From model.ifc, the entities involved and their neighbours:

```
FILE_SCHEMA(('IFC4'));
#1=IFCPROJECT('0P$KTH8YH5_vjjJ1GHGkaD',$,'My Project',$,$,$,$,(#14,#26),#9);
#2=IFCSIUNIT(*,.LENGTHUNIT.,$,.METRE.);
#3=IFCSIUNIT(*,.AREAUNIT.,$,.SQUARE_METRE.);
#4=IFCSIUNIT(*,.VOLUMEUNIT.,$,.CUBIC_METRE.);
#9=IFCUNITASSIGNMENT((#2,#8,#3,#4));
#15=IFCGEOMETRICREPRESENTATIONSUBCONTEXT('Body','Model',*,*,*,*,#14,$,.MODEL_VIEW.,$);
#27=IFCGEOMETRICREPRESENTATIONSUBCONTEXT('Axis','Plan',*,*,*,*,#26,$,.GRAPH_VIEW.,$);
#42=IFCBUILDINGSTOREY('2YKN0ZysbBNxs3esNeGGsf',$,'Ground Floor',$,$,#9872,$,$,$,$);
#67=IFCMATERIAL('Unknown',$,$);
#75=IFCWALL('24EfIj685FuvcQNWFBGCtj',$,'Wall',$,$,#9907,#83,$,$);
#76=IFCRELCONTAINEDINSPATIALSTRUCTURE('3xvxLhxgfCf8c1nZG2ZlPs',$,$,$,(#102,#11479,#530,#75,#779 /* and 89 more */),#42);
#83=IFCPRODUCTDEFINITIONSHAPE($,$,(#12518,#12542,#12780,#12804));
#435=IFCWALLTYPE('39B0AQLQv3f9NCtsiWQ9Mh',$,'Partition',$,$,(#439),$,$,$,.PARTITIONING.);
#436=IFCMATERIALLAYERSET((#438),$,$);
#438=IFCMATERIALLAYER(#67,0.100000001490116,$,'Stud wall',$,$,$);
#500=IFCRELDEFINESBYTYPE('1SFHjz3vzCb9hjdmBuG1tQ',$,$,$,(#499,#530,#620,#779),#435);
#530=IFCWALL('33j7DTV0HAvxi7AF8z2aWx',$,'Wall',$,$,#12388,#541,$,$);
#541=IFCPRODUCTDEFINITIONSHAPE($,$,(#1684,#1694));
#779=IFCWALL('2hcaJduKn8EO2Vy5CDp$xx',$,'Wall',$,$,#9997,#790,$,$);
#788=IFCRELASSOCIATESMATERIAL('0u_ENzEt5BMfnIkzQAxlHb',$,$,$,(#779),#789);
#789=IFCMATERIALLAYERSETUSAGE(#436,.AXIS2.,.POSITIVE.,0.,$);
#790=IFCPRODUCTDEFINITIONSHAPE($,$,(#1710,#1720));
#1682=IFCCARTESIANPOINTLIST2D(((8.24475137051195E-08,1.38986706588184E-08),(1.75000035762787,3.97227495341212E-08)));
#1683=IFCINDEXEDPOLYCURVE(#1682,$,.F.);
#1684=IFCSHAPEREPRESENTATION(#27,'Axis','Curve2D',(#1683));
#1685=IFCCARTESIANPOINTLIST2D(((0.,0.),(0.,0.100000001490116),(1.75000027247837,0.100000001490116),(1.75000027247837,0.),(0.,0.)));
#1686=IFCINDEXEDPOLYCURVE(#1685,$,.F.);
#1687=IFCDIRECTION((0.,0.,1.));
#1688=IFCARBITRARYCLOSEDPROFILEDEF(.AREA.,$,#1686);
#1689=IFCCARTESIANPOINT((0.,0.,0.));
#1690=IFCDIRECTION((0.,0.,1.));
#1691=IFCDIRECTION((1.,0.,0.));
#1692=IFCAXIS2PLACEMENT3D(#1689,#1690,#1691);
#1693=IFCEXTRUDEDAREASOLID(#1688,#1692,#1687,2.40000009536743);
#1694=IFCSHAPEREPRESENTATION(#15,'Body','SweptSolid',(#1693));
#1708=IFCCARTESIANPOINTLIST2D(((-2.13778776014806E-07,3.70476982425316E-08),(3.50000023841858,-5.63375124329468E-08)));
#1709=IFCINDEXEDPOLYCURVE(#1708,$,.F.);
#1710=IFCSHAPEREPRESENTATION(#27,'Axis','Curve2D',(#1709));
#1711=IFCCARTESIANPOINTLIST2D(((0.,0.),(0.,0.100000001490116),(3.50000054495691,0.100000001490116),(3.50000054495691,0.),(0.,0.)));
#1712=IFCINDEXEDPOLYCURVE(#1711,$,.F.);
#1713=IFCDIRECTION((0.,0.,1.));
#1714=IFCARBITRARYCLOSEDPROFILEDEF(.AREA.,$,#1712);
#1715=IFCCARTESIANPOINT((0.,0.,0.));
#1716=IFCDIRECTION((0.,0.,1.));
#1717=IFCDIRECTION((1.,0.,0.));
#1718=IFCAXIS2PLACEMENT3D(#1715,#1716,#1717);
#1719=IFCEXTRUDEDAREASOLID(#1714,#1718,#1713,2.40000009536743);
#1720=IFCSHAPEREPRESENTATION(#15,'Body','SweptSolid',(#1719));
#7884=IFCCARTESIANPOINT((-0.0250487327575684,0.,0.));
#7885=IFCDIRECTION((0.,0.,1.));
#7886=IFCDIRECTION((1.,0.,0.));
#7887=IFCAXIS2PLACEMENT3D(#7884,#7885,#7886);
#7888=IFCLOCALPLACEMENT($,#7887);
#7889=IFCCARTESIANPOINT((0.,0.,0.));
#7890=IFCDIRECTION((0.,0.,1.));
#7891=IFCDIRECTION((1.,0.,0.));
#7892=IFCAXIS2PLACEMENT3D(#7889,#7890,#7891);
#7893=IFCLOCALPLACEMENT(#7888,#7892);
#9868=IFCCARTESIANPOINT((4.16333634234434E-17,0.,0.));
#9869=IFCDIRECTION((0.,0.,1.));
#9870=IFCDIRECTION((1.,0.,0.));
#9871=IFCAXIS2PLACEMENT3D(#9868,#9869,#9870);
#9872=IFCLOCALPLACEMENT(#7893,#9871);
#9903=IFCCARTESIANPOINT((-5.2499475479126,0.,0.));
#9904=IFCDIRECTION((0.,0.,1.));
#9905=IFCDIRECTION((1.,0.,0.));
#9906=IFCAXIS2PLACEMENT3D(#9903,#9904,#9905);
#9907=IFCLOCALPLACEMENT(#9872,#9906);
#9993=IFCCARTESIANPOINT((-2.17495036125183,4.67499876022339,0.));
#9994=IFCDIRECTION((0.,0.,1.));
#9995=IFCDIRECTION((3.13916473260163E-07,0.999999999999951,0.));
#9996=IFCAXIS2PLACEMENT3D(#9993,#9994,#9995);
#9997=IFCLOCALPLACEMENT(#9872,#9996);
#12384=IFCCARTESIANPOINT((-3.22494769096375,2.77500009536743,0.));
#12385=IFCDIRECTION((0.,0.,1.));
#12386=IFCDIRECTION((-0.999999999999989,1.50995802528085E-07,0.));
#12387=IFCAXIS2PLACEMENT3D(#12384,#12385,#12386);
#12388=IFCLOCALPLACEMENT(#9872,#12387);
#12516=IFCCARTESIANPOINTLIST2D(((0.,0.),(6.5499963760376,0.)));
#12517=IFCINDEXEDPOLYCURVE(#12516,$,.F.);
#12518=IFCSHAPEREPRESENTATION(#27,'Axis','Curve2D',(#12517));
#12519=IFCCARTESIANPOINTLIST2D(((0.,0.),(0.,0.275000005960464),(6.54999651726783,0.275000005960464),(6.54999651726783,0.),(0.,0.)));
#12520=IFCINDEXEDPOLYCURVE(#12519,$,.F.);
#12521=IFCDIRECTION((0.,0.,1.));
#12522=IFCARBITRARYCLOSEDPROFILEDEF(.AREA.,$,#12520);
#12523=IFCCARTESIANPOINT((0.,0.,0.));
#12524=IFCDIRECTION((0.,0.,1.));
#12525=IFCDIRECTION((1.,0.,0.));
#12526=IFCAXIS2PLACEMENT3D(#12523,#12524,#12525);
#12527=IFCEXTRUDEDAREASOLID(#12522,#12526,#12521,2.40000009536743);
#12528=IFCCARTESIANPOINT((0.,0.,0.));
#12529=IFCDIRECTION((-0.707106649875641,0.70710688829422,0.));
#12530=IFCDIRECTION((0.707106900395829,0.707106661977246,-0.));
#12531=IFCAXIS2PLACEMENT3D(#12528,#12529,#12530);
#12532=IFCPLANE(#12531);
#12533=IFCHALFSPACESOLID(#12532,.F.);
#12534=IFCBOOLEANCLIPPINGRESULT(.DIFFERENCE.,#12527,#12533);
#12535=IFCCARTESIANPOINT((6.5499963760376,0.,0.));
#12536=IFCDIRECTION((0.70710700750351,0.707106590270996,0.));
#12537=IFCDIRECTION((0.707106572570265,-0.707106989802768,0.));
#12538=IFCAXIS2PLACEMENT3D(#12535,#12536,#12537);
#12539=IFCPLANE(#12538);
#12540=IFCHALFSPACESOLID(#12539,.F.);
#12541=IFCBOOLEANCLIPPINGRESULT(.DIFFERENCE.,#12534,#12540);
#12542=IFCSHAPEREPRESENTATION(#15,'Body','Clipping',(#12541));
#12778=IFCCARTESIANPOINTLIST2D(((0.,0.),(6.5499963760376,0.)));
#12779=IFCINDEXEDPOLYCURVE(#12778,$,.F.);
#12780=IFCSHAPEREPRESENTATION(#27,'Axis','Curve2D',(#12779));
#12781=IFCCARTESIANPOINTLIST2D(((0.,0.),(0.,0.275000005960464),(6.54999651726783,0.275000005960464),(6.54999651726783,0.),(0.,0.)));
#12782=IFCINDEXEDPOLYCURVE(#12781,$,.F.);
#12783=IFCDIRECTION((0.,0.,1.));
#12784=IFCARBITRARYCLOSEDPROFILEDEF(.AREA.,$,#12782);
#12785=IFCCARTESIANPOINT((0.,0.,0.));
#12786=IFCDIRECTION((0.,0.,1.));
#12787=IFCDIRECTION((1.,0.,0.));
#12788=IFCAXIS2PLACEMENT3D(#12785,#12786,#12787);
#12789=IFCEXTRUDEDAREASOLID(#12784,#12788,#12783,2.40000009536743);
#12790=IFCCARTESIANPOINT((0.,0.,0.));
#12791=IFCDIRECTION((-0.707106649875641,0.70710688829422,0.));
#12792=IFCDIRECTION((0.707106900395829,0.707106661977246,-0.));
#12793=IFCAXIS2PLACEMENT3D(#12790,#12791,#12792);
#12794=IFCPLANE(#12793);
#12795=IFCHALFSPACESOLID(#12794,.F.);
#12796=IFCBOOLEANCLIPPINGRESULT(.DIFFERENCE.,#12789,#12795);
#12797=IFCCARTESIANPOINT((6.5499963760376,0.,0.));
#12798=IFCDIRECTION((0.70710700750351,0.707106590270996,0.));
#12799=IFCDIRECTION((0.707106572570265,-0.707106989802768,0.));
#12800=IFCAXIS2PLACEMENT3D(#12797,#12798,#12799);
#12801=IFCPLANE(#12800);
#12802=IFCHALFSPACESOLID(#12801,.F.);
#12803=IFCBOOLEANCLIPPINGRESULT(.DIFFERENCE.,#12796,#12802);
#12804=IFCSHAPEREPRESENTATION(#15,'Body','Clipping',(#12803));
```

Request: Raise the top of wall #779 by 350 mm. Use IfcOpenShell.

```python
import ifcopenshell
import ifcopenshell.geom
import ifcopenshell.util.representation
import ifcopenshell.util.shape
import ifcopenshell.util.unit

model = ifcopenshell.open("model.ifc")
unit_scale = ifcopenshell.util.unit.calculate_unit_scale(model)
settings = ifcopenshell.geom.settings()


def volume(element):
    """Net volume in cubic metres, openings subtracted."""
    shape = ifcopenshell.geom.create_shape(settings, element)
    return ifcopenshell.util.shape.get_volume(shape.geometry)


wall = model.by_guid("2hcaJduKn8EO2Vy5CDp$xx")
before = volume(wall)

body = ifcopenshell.util.representation.get_representation(wall, "Model", "Body")
solid = body.Items[0]
old_height = solid.Depth
solid.Depth += 0.35 / unit_scale
after = volume(wall)

print(f"height {old_height:g} -> {solid.Depth:g}, volume {before:.3f} -> {after:.3f} m3")

model.write("model-out.ifc")
```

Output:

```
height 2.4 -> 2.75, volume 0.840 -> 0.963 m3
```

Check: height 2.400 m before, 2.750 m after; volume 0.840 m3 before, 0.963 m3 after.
